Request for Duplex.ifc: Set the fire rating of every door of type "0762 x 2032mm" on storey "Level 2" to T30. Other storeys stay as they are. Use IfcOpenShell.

First a look at what the model holds.

```python
import ifcopenshell
import ifcopenshell.util.element

model = ifcopenshell.open("Duplex.ifc")
print(model.schema)
storey = next(s for s in model.by_type("IfcBuildingStorey") if s.Name == "Level 2")
doors = [e for e in ifcopenshell.util.element.get_decomposition(storey) if e.is_a("IfcDoor")]
seen = {}
for e in doors:
    element_type = ifcopenshell.util.element.get_type(e)
    key = (element_type.Name if element_type != e and element_type else None, ifcopenshell.util.element.get_pset(e, "Pset_DoorCommon", "FireRating"))
    seen[key] = seen.get(key, 0) + 1
for (name, value), count in sorted(seen.items(), key=str):
    print(count, "x", name, "|", value)
```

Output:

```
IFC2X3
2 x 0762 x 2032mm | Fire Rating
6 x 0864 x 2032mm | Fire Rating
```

```python
import ifcopenshell
import ifcopenshell.api.pset
import ifcopenshell.util.element

model = ifcopenshell.open("Duplex.ifc")

storey = next(s for s in model.by_type("IfcBuildingStorey") if s.Name == "Level 2")
doors = [e for e in ifcopenshell.util.element.get_decomposition(storey) if e.is_a("IfcDoor")]

count = 0
for e in doors:
    element_type = ifcopenshell.util.element.get_type(e)
    if element_type in (None, e) or element_type.Name != "0762 x 2032mm":
        continue
    # add_pset returns the element's existing set when there is one.
    pset = ifcopenshell.api.pset.add_pset(model, product=e, name="Pset_DoorCommon")
    ifcopenshell.api.pset.edit_pset(model, pset=pset, properties={"FireRating": "T30"})
    count += 1

print(count, "doors updated")

model.write("Duplex_v2.ifc")
```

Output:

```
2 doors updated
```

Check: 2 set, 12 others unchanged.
